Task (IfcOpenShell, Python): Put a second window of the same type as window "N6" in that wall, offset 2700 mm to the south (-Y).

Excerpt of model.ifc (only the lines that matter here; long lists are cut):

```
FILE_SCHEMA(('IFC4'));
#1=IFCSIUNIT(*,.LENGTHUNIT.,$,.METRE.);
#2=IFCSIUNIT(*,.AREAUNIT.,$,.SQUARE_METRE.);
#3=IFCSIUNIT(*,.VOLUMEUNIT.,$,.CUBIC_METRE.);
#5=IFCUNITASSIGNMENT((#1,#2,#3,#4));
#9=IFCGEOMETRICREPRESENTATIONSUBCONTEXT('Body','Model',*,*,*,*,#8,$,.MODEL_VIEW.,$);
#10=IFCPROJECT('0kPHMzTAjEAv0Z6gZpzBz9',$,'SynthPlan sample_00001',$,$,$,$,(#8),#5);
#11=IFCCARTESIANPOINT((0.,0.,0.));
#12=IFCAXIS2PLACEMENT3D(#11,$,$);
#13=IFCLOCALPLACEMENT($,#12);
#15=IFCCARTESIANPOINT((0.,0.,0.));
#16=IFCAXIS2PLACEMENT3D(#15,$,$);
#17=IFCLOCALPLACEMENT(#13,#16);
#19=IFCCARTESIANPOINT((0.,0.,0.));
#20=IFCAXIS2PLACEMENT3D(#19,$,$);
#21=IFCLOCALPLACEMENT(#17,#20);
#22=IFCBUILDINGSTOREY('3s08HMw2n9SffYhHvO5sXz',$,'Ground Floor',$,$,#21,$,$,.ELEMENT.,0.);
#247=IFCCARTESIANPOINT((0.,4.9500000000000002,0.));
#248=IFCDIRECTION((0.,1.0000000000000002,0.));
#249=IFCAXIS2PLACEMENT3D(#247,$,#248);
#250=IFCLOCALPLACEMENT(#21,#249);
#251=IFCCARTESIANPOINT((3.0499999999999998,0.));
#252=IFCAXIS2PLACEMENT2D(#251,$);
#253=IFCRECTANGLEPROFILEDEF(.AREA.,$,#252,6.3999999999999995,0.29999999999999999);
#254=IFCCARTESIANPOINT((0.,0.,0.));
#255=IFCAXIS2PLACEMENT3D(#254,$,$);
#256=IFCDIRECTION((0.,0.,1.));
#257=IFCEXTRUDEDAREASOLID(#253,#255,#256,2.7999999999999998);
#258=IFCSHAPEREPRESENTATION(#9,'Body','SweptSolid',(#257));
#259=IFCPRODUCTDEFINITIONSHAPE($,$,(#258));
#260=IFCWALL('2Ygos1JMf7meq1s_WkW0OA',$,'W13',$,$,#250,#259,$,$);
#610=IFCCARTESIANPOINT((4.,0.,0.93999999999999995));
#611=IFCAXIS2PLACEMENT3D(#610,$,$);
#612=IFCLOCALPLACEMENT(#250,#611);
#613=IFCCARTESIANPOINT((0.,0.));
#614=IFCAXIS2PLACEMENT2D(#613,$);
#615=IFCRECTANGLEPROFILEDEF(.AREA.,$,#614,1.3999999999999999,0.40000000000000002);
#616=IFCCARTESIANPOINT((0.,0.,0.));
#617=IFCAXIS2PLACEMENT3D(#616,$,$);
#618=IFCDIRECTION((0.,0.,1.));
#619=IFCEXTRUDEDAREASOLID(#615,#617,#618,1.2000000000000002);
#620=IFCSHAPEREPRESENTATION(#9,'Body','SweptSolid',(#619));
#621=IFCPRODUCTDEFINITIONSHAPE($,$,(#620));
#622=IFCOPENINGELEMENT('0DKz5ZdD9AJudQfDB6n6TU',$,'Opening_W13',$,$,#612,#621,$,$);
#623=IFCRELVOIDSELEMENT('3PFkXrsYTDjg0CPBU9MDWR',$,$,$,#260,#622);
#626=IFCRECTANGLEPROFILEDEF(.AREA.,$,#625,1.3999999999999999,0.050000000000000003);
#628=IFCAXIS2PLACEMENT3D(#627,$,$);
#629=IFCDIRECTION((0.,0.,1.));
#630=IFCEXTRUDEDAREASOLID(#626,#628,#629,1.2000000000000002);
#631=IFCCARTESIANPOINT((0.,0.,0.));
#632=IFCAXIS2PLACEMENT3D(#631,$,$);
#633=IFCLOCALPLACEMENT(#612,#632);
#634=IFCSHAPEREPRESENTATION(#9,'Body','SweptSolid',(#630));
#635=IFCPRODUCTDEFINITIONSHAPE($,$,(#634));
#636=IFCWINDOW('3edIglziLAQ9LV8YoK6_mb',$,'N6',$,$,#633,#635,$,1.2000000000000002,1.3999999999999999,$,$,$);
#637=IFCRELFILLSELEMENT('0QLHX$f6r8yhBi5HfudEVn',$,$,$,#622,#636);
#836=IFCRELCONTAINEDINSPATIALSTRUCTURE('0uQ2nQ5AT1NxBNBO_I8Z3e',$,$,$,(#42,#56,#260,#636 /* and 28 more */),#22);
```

```python
import ifcopenshell
import ifcopenshell.api.feature
import ifcopenshell.api.geometry
import ifcopenshell.api.root
import ifcopenshell.geom
import ifcopenshell.util.element
import ifcopenshell.util.placement
import ifcopenshell.util.shape

model = ifcopenshell.open("model.ifc")
settings = ifcopenshell.geom.settings()


def volume(element):
    """Net volume in cubic metres, openings subtracted."""
    shape = ifcopenshell.geom.create_shape(settings, element)
    return ifcopenshell.util.shape.get_volume(shape.geometry)


window = model.by_guid("3edIglziLAQ9LV8YoK6_mb")
opening = window.FillsVoids[0].RelatingOpeningElement
wall = opening.VoidsElements[0].RelatingBuildingElement
before = volume(wall)
shift = ifcopenshell.util.placement.get_local_placement(wall.ObjectPlacement)[:3, 0] * -2.7

# copy_class copies the void relationship, type, container and properties, but no geometry.
new_opening = ifcopenshell.api.root.copy_class(model, product=opening)
new_opening.Representation = ifcopenshell.util.element.copy_deep(
    model, opening.Representation, exclude=["IfcGeometricRepresentationContext", "IfcRepresentationMap"]
)
new_window = ifcopenshell.api.root.copy_class(model, product=window)
new_window.Representation = ifcopenshell.util.element.copy_deep(
    model, window.Representation, exclude=["IfcGeometricRepresentationContext", "IfcRepresentationMap"]
)
ifcopenshell.api.feature.add_filling(model, opening=new_opening, element=new_window)

for old, new in ((opening, new_opening), (window, new_window)):
    matrix = ifcopenshell.util.placement.get_local_placement(old.ObjectPlacement)
    matrix[:3, 3] += shift
    ifcopenshell.api.geometry.edit_object_placement(model, product=new, matrix=matrix, is_si=False)

after = volume(wall)

print(f"wall volume {before:.3f} -> {after:.3f} m3")

model.write("model-out.ifc")
```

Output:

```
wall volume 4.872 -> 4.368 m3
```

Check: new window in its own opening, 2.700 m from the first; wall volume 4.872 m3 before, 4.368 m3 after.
